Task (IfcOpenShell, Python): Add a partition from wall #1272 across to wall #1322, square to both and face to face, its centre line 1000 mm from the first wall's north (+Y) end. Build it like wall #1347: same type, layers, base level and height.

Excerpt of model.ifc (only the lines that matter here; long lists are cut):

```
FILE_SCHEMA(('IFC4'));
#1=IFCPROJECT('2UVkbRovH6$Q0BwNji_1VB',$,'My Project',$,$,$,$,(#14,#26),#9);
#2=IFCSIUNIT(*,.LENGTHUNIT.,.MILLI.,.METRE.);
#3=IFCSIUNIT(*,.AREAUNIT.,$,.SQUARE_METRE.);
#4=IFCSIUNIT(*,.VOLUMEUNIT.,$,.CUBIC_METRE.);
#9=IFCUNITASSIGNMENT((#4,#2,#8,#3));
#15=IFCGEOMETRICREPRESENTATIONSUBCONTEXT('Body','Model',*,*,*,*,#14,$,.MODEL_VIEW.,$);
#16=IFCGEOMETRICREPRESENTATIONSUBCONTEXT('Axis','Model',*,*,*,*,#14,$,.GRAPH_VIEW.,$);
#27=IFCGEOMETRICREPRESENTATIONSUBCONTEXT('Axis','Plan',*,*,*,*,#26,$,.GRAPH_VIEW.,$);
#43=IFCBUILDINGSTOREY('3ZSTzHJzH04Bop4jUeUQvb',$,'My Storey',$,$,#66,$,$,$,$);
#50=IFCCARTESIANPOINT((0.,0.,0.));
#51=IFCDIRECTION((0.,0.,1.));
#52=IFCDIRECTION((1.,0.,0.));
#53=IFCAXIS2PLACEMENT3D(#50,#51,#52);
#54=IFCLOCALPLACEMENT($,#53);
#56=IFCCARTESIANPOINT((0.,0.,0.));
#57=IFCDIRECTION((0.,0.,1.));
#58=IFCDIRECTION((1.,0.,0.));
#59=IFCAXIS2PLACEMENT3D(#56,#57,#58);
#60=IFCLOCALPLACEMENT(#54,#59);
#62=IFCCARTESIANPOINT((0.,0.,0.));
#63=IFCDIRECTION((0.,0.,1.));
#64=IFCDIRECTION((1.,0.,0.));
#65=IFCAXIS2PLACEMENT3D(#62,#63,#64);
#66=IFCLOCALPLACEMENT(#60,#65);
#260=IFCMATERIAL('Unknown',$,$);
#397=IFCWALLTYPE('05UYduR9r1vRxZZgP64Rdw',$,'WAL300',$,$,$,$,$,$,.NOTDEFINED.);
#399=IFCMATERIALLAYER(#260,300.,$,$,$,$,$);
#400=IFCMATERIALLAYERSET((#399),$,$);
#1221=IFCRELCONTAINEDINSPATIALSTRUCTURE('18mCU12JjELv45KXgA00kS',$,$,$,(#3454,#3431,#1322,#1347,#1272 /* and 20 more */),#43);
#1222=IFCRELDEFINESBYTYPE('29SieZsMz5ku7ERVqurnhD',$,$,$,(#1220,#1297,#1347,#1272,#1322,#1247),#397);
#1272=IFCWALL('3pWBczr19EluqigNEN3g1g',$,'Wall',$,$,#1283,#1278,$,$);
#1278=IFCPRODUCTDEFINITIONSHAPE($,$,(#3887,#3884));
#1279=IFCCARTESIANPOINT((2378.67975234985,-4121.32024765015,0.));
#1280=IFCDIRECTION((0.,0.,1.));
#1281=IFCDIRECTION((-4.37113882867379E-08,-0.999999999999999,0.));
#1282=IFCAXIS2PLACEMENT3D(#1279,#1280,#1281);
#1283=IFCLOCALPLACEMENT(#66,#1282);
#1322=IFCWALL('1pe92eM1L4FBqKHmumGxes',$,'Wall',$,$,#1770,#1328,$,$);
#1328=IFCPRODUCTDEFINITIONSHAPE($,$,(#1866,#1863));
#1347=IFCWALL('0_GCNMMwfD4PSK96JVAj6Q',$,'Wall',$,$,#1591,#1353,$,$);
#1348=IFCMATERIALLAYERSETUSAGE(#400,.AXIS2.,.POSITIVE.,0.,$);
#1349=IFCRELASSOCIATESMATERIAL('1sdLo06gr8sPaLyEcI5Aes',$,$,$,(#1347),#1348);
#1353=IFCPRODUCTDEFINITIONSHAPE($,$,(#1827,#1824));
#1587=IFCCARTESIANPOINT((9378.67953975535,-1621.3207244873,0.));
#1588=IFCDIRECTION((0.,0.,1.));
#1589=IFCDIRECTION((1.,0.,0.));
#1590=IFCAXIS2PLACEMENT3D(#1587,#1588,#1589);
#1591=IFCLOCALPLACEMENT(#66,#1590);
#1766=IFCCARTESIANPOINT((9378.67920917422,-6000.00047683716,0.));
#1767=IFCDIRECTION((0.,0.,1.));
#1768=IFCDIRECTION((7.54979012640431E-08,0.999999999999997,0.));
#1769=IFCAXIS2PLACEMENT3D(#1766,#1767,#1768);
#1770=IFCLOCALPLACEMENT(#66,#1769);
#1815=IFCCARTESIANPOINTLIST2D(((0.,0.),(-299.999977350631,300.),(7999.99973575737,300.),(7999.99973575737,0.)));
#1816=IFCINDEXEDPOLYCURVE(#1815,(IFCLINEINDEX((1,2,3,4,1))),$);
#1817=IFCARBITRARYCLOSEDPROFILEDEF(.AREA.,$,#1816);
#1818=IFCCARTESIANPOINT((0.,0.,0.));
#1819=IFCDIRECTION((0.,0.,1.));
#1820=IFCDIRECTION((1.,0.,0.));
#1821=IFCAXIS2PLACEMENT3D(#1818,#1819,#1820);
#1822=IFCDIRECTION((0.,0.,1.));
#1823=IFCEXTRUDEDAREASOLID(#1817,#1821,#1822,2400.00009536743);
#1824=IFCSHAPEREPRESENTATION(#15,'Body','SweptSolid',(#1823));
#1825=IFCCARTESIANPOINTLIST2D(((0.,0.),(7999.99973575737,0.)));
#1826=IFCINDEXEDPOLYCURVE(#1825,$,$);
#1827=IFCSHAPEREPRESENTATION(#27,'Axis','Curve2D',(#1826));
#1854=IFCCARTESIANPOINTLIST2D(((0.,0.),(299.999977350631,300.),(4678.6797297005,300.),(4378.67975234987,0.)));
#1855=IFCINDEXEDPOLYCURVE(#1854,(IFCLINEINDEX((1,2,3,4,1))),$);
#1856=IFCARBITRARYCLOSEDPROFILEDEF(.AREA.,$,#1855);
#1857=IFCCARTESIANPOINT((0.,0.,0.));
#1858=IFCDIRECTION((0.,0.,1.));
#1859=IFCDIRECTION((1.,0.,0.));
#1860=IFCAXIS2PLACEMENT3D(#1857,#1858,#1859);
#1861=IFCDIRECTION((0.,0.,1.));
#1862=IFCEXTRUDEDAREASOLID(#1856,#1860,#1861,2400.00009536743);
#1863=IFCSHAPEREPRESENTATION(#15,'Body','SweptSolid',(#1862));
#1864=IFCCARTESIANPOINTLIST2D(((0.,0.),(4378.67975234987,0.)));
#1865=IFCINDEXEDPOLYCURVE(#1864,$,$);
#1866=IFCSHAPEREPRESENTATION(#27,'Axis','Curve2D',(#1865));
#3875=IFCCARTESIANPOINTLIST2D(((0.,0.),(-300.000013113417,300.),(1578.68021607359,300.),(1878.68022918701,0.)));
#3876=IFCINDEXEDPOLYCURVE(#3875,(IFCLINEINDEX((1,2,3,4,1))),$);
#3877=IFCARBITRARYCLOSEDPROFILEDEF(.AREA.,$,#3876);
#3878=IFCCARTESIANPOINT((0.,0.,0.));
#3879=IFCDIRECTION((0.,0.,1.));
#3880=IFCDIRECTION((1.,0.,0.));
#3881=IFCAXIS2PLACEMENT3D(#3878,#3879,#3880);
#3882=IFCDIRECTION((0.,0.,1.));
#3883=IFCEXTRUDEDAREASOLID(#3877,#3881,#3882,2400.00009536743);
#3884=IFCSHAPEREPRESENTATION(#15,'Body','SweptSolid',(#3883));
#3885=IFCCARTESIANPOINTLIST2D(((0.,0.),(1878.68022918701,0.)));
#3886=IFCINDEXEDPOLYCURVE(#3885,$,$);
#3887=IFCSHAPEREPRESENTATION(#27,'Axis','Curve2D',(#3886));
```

```python
import numpy as np
import ifcopenshell
import ifcopenshell.api.geometry
import ifcopenshell.api.material
import ifcopenshell.api.pset
import ifcopenshell.api.root
import ifcopenshell.api.spatial
import ifcopenshell.api.type
import ifcopenshell.geom
import ifcopenshell.util.element
import ifcopenshell.util.placement
import ifcopenshell.util.representation
import ifcopenshell.util.shape
import ifcopenshell.util.unit

model = ifcopenshell.open("model.ifc")
unit_scale = ifcopenshell.util.unit.calculate_unit_scale(model)
settings = ifcopenshell.geom.settings()
settings.set("use-world-coords", True)

start_wall = model.by_guid("3pWBczr19EluqigNEN3g1g")
end_wall = model.by_guid("1pe92eM1L4FBqKHmumGxes")
like = model.by_guid("0_GCNMMwfD4PSK96JVAj6Q")
matrix = ifcopenshell.util.placement.get_local_placement(start_wall.ObjectPlacement)
matrix[:3, 3] *= unit_scale


def extent(element):
    """Bounding box in the first wall's axes, in metres."""
    shape = ifcopenshell.geom.create_shape(settings, element)
    points = (ifcopenshell.util.shape.get_vertices(shape.geometry) - matrix[:3, 3]) @ matrix[:3, :3]
    return points.min(axis=0), points.max(axis=0)


y_start = extent(start_wall)[1][1]
y_end = extent(end_wall)[0][1]
like_min, like_max = extent(like)
length, height = float(abs(y_end - y_start)), float(like_max[2] - like_min[2])
layer_set = ifcopenshell.util.element.get_material(like, should_skip_usage=True)
thickness = sum(layer.LayerThickness for layer in layer_set.MaterialLayers) * unit_scale

wall = ifcopenshell.api.root.create_entity(model, ifc_class="IfcWall", name="New partition")
storey = ifcopenshell.util.element.get_container(like)
ifcopenshell.api.spatial.assign_container(model, products=[wall], relating_structure=storey)
ifcopenshell.api.type.assign_type(
    model, related_objects=[wall], relating_type=ifcopenshell.util.element.get_type(like), should_map_representations=False
)
rel = ifcopenshell.api.material.assign_material(
    model, products=[wall], type="IfcMaterialLayerSetUsage", material=layer_set
)
rel.RelatingMaterial.OffsetFromReferenceLine = -thickness / 2 / unit_scale
pset = ifcopenshell.api.pset.add_pset(model, product=wall, name="Pset_WallCommon")
ifcopenshell.api.pset.edit_pset(model, pset=pset, properties={"IsExternal": False, "LoadBearing": False})

# The axis runs down the middle of the wall.
axis = ifcopenshell.api.geometry.add_axis_representation(
    model, context=ifcopenshell.util.representation.get_context(model, "Model", "Axis"), axis=[(0.0, 0.0), (length, 0.0)]
)
body = ifcopenshell.api.geometry.add_wall_representation(
    model,
    context=ifcopenshell.util.representation.get_context(model, "Model", "Body", "MODEL_VIEW"),
    length=length,
    height=height,
    thickness=thickness,
    offset=-thickness / 2,
)
for representation in (axis, body):
    ifcopenshell.api.geometry.assign_representation(model, product=wall, representation=representation)

placement = matrix @ ifcopenshell.util.placement.rotation(90, "Z")
placement[:, 3] = matrix @ np.array([extent(start_wall)[0][0] + 1, y_start, like_min[2], 1.0])
ifcopenshell.api.geometry.edit_object_placement(model, product=wall, matrix=placement)

print(f"partition {length:.3f} m long, {height:.3f} m high, {thickness:.3f} m thick")

model.write("model_edited.ifc")
```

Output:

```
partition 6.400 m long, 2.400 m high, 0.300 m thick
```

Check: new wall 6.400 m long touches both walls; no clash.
